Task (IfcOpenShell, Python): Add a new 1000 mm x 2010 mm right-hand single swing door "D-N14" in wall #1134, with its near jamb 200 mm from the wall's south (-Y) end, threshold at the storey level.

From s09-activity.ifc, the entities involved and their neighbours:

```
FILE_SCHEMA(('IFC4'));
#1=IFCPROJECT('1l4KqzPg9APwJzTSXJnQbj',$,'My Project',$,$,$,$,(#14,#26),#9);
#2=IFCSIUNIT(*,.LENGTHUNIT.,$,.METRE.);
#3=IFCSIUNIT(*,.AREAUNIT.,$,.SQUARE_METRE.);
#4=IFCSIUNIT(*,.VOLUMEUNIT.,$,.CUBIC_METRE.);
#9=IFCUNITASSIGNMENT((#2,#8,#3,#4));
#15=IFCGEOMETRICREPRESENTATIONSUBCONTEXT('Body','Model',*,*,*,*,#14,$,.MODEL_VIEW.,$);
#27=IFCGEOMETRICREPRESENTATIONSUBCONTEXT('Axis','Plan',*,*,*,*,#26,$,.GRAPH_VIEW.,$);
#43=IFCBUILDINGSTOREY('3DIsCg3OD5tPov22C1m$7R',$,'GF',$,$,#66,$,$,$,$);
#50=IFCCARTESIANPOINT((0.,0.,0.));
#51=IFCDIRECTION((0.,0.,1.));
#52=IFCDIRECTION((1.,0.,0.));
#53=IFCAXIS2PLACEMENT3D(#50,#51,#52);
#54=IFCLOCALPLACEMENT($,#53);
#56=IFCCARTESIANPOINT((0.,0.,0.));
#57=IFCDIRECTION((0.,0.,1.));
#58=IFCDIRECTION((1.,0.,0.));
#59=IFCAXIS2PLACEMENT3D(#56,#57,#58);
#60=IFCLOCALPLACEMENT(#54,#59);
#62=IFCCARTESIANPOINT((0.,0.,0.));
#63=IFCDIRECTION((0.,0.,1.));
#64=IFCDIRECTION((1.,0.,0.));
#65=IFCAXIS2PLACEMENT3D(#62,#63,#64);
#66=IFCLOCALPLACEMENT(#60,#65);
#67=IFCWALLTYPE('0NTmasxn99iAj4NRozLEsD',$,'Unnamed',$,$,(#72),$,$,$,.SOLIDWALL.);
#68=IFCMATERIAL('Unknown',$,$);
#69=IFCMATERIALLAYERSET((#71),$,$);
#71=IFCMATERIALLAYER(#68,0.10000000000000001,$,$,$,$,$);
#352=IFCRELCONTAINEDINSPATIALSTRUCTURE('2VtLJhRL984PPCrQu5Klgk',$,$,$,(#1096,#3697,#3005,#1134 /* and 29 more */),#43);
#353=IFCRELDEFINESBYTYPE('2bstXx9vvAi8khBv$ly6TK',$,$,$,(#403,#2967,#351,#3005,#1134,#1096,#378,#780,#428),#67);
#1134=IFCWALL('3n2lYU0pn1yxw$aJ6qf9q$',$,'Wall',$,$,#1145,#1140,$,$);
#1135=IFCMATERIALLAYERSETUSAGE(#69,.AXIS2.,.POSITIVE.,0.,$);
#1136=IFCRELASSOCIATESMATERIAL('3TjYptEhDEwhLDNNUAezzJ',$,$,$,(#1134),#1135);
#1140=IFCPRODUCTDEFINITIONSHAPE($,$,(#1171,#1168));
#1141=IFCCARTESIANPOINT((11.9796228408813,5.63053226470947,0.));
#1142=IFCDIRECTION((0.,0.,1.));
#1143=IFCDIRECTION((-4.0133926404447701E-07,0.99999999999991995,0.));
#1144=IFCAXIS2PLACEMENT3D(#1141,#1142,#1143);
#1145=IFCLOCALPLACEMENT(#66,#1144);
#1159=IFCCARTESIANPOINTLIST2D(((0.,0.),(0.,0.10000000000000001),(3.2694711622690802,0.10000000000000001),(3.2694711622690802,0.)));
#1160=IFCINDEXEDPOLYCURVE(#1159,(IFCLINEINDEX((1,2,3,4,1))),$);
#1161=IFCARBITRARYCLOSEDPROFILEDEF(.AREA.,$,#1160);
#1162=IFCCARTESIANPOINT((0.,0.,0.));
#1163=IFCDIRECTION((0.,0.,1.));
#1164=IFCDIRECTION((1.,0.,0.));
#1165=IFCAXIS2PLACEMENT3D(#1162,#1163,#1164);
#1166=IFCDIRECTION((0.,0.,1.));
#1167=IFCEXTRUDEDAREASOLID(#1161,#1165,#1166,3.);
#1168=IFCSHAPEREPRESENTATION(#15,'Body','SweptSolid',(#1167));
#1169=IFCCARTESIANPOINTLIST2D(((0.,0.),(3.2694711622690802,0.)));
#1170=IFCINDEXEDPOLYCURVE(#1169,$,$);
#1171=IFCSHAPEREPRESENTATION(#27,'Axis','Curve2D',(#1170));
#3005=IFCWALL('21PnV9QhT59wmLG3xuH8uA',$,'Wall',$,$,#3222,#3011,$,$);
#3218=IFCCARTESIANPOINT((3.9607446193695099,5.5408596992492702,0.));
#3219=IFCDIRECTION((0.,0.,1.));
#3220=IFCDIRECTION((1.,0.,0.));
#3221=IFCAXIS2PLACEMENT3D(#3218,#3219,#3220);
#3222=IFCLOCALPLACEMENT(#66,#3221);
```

```python
import numpy as np
import ifcopenshell
import ifcopenshell.api.feature
import ifcopenshell.api.geometry
import ifcopenshell.api.root
import ifcopenshell.api.spatial
import ifcopenshell.geom
import ifcopenshell.util.element
import ifcopenshell.util.placement
import ifcopenshell.util.representation
import ifcopenshell.util.shape
import ifcopenshell.util.unit

model = ifcopenshell.open("s09-activity.ifc")
unit_scale = ifcopenshell.util.unit.calculate_unit_scale(model)
settings = ifcopenshell.geom.settings()


def volume(element):
    """Net volume in cubic metres, openings subtracted."""
    shape = ifcopenshell.geom.create_shape(settings, element)
    return ifcopenshell.util.shape.get_volume(shape.geometry)


wall = model.by_guid("3n2lYU0pn1yxw$aJ6qf9q$")
storey = ifcopenshell.util.element.get_container(wall, ifc_class="IfcBuildingStorey")
context = ifcopenshell.util.representation.get_context(model, "Model", "Body", "MODEL_VIEW")
before = volume(wall)

width, height, from_end, sill = 1, 2.01, 0.2, 0.0  # metres

# The wall runs along its own X axis, and the end named is its -X end.
wall_shape = ifcopenshell.geom.create_shape(settings, wall)
x, y, z = ifcopenshell.util.shape.get_vertices(wall_shape.geometry).T
start = x.min() + from_end
face, thickness = float(y.min()), float(y.max() - y.min())
wall_matrix = ifcopenshell.util.placement.get_local_placement(wall.ObjectPlacement)
level = ifcopenshell.util.placement.get_local_placement(storey.ObjectPlacement)[2, 3]


def in_wall(x, y):
    """Placement at x, y metres in the wall's axes, at sill height."""
    matrix = wall_matrix.copy()
    matrix[:, 3] = wall_matrix @ np.array([x / unit_scale, y / unit_scale, 0.0, 1.0])
    matrix[2, 3] = level + sill / unit_scale
    return matrix


# Opening: a box that overshoots both wall faces by 50 mm.
opening = ifcopenshell.api.root.create_entity(model, ifc_class="IfcOpeningElement", predefined_type="OPENING")
box = ifcopenshell.api.geometry.add_wall_representation(
    model, context=context, length=width, height=height, thickness=thickness + 0.1
)
ifcopenshell.api.geometry.assign_representation(model, product=opening, representation=box)
ifcopenshell.api.geometry.edit_object_placement(model, product=opening, matrix=in_wall(start, face - 0.05), is_si=False)
ifcopenshell.api.feature.add_feature(model, feature=opening, element=wall)

door = ifcopenshell.api.root.create_entity(model, ifc_class="IfcDoor", name="D-N14", predefined_type="DOOR")
door.OverallWidth, door.OverallHeight = width / unit_scale, height / unit_scale
door.OperationType = "SINGLE_SWING_RIGHT"
body = ifcopenshell.api.geometry.add_door_representation(
    model,
    context=context,
    overall_width=door.OverallWidth,
    overall_height=door.OverallHeight,
    operation_type="SINGLE_SWING_RIGHT",
    lining_properties={"LiningDepth": thickness / unit_scale, "ThresholdDepth": thickness / unit_scale},
)
ifcopenshell.api.geometry.assign_representation(model, product=door, representation=body)
ifcopenshell.api.spatial.assign_container(model, products=[door], relating_structure=storey)
ifcopenshell.api.feature.add_filling(model, opening=opening, element=door)

# The lining spans the wall, so the door starts at the wall face.
ifcopenshell.api.geometry.edit_object_placement(model, product=door, matrix=in_wall(start, face), is_si=False)

after = volume(wall)

print(f"wall volume {before:.3f} -> {after:.3f} m3")

model.write("s09-activity_updated.ifc")
```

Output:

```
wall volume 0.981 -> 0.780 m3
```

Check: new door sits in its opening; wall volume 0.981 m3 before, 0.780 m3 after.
